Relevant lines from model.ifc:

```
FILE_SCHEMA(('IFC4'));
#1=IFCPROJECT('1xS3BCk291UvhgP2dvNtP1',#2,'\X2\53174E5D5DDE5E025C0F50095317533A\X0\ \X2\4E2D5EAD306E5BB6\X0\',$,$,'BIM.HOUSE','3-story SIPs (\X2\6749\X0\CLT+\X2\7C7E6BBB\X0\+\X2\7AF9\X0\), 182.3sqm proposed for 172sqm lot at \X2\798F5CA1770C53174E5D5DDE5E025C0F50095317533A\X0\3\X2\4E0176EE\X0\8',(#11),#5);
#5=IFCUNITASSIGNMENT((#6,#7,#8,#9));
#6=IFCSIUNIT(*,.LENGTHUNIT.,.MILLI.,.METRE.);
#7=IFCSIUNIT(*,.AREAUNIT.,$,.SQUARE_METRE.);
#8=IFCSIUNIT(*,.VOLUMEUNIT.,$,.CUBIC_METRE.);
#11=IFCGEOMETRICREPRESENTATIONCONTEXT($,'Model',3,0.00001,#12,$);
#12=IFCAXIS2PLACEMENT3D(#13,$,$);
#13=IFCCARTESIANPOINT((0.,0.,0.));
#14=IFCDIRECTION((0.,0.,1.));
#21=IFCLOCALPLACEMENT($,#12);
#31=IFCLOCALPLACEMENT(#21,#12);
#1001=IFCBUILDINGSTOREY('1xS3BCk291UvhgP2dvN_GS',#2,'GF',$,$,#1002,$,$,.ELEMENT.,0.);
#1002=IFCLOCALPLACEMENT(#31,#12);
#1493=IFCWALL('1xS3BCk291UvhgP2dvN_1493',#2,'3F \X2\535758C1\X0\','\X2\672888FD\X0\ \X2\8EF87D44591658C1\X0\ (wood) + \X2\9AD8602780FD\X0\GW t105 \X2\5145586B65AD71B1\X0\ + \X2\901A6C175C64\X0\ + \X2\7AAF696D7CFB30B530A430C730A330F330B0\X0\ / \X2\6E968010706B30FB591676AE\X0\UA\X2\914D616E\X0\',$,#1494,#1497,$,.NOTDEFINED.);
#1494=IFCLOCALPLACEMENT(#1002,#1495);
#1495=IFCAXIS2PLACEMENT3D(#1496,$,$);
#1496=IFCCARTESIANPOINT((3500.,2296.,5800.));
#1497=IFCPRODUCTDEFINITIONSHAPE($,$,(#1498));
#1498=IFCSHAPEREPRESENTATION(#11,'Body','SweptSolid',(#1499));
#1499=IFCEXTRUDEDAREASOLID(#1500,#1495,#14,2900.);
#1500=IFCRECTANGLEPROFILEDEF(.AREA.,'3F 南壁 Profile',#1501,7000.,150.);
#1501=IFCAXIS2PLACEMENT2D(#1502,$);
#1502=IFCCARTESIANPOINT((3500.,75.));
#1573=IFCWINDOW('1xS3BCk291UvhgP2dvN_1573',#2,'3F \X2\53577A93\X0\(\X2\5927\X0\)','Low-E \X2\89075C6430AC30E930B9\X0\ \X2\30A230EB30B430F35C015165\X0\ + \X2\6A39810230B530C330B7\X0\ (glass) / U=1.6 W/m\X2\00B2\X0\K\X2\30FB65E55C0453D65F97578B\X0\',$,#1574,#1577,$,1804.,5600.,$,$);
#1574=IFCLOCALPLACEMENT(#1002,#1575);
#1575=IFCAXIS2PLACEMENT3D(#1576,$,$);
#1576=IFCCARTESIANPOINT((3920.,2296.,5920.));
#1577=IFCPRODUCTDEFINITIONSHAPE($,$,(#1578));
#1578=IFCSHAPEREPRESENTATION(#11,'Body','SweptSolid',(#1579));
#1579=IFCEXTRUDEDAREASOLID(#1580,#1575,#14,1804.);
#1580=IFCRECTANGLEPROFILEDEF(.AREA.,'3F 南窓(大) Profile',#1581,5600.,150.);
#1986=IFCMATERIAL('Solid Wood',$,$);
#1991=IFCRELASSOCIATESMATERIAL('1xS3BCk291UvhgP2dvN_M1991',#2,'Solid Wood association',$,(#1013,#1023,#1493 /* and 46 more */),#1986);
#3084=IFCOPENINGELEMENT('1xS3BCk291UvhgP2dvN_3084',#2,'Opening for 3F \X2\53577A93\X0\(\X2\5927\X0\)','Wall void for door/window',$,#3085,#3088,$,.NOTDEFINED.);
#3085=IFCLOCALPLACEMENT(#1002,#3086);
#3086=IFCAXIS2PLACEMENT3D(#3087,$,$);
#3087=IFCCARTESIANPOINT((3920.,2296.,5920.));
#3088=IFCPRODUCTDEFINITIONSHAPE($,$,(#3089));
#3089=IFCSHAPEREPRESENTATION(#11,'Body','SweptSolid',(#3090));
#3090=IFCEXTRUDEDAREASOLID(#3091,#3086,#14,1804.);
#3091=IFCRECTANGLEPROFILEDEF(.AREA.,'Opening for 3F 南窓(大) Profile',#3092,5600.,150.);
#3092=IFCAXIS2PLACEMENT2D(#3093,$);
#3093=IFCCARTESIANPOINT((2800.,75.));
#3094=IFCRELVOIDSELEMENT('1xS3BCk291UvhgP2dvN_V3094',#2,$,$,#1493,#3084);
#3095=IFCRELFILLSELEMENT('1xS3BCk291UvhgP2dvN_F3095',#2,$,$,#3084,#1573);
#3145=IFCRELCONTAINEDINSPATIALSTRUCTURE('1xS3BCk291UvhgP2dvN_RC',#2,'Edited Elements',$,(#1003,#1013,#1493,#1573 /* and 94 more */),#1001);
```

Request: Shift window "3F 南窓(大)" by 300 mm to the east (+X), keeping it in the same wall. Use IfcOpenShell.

```python
import ifcopenshell
import ifcopenshell.api.geometry
import ifcopenshell.util.placement

model = ifcopenshell.open("model.ifc")

window = model.by_guid("1xS3BCk291UvhgP2dvN_1573")
opening = window.FillsVoids[0].RelatingOpeningElement
wall = opening.VoidsElements[0].RelatingBuildingElement

wall_matrix = ifcopenshell.util.placement.get_local_placement(wall.ObjectPlacement)
shift = wall_matrix[:3, 0] * 300.0
before = ifcopenshell.util.placement.get_local_placement(window.ObjectPlacement)[:3, 3].copy()

# The window is not placed relative to its opening, so move both.
for product in (opening, window):
    matrix = ifcopenshell.util.placement.get_local_placement(product.ObjectPlacement)
    matrix[:3, 3] += shift
    ifcopenshell.api.geometry.edit_object_placement(model, product=product, matrix=matrix, is_si=False)

after = ifcopenshell.util.placement.get_local_placement(window.ObjectPlacement)[:3, 3]
print("window moved by", (after - before).round(3) + 0.0)

model.write("model_v2.ifc")
```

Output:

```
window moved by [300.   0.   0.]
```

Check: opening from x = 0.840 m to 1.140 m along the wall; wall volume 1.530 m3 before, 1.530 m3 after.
